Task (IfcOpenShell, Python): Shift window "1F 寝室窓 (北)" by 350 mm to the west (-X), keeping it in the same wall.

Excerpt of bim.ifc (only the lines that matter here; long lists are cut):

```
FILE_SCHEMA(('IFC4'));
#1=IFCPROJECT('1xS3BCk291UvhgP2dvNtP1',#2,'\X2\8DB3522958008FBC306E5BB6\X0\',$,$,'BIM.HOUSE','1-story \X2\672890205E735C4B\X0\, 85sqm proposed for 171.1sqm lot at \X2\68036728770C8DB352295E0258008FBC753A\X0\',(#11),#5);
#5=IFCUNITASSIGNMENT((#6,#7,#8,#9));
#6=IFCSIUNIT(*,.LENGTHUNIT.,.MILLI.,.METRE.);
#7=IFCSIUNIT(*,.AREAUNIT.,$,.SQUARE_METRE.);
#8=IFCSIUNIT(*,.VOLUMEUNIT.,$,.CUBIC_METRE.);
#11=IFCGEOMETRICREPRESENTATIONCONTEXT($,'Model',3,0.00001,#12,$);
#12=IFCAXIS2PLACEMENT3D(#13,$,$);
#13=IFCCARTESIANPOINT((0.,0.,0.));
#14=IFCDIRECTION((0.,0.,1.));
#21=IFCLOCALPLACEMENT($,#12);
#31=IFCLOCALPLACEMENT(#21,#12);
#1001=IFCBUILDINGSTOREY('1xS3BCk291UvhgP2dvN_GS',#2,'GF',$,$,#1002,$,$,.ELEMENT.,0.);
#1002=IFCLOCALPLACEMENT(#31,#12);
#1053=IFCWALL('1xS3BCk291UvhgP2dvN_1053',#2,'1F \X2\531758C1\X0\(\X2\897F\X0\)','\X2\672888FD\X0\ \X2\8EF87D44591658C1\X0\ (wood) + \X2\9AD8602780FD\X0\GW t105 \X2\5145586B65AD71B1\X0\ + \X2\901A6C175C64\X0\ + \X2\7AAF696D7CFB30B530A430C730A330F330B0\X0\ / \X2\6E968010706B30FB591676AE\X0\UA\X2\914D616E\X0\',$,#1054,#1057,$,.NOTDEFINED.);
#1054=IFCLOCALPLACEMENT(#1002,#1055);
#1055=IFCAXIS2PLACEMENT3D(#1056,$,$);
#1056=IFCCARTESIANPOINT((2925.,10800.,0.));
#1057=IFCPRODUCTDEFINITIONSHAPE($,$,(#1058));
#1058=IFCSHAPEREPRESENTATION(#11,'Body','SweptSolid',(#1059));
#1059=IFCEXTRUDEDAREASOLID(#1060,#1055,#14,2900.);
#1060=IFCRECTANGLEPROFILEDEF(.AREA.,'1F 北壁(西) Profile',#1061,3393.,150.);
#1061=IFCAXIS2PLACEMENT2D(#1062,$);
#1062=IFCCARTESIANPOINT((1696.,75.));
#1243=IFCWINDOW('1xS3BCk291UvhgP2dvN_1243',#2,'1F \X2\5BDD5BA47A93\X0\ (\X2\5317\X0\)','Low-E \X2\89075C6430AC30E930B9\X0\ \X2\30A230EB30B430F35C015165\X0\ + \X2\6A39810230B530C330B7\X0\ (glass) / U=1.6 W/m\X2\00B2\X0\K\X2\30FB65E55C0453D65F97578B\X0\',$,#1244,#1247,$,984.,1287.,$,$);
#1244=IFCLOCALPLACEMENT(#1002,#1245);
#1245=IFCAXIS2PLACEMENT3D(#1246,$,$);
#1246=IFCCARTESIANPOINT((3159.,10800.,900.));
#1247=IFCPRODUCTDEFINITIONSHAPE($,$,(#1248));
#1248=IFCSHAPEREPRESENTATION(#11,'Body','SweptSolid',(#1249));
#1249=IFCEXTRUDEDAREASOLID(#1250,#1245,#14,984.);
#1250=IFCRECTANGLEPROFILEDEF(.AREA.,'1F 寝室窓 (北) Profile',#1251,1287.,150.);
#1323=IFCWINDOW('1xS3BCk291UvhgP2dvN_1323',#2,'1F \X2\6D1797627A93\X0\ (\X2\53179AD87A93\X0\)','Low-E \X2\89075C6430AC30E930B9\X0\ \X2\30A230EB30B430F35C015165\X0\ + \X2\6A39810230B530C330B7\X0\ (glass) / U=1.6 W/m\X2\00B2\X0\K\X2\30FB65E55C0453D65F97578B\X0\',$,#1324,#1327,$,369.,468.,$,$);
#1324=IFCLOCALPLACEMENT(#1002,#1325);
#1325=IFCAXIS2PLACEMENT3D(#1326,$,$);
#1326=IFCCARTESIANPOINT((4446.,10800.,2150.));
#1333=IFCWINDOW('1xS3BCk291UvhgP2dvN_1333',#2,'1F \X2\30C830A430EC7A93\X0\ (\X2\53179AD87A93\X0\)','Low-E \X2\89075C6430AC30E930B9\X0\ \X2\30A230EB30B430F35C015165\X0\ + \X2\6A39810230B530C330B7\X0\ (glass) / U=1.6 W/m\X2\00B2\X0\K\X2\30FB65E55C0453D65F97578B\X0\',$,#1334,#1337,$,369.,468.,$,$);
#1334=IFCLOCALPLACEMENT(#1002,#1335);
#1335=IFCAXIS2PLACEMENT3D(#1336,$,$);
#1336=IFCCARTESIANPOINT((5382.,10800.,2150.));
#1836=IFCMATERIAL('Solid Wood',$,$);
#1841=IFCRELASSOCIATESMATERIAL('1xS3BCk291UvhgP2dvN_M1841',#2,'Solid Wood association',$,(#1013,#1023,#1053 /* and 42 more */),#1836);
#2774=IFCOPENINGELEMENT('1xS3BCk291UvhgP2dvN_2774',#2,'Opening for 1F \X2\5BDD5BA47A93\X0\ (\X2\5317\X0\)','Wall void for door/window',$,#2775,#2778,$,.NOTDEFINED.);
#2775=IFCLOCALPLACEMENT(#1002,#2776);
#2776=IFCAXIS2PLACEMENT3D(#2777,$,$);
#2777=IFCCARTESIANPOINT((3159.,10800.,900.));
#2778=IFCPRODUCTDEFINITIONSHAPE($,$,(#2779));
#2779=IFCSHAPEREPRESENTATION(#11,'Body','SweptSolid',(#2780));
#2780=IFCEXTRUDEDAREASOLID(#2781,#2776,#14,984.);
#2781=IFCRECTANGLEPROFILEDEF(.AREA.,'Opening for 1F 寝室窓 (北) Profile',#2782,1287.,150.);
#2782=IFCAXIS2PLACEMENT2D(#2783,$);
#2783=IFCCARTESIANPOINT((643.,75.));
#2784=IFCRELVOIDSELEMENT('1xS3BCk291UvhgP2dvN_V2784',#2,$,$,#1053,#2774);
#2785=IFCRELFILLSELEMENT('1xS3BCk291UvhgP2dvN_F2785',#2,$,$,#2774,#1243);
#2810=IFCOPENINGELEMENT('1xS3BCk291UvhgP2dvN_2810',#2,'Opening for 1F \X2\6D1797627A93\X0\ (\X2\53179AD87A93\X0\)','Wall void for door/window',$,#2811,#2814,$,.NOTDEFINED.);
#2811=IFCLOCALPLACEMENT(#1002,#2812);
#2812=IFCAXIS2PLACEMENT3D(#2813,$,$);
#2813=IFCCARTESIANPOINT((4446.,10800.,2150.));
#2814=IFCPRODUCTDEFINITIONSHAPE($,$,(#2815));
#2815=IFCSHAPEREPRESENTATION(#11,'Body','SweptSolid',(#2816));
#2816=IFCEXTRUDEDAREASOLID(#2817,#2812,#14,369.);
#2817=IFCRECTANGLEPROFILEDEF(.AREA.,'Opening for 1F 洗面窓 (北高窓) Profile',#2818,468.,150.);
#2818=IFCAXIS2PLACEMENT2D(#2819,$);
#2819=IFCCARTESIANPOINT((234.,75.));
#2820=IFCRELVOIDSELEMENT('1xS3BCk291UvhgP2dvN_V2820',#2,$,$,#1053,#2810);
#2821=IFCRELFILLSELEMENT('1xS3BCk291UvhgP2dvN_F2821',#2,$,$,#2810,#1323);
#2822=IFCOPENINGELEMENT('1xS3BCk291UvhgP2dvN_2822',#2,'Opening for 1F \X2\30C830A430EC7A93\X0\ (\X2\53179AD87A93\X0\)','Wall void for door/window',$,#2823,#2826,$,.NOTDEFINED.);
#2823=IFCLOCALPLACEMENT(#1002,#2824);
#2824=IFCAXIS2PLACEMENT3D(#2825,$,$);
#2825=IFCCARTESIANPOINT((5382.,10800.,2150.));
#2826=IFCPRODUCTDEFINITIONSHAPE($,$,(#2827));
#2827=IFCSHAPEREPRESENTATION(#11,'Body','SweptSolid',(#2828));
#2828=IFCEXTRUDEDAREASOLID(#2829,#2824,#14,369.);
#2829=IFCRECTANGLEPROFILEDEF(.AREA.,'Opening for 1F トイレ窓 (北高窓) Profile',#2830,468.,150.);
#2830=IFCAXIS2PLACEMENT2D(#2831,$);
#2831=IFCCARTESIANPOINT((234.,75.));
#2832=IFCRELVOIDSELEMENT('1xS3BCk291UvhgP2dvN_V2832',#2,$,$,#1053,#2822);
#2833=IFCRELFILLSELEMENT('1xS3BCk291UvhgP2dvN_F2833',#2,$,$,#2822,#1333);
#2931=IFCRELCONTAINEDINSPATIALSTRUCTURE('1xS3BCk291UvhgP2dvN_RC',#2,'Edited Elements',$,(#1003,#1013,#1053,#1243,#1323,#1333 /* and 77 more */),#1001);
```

```python
import ifcopenshell
import ifcopenshell.api.geometry
import ifcopenshell.util.placement
import ifcopenshell.util.unit

model = ifcopenshell.open("bim.ifc")
unit_scale = ifcopenshell.util.unit.calculate_unit_scale(model)

window = model.by_guid("1xS3BCk291UvhgP2dvN_1243")
opening = window.FillsVoids[0].RelatingOpeningElement
wall = opening.VoidsElements[0].RelatingBuildingElement

wall_matrix = ifcopenshell.util.placement.get_local_placement(wall.ObjectPlacement)
shift = wall_matrix[:3, 0] * -0.35 / unit_scale
before = ifcopenshell.util.placement.get_local_placement(window.ObjectPlacement)[:3, 3].copy()

# The window is not placed relative to its opening, so move both.
for product in (opening, window):
    matrix = ifcopenshell.util.placement.get_local_placement(product.ObjectPlacement)
    matrix[:3, 3] += shift
    ifcopenshell.api.geometry.edit_object_placement(model, product=product, matrix=matrix, is_si=False)

after = ifcopenshell.util.placement.get_local_placement(window.ObjectPlacement)[:3, 3]
print("window moved by", (after - before).round(3) + 0.0)

model.write("bim-out.ifc")
```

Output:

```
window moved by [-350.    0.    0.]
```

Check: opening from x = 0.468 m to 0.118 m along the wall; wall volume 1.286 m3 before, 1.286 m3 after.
